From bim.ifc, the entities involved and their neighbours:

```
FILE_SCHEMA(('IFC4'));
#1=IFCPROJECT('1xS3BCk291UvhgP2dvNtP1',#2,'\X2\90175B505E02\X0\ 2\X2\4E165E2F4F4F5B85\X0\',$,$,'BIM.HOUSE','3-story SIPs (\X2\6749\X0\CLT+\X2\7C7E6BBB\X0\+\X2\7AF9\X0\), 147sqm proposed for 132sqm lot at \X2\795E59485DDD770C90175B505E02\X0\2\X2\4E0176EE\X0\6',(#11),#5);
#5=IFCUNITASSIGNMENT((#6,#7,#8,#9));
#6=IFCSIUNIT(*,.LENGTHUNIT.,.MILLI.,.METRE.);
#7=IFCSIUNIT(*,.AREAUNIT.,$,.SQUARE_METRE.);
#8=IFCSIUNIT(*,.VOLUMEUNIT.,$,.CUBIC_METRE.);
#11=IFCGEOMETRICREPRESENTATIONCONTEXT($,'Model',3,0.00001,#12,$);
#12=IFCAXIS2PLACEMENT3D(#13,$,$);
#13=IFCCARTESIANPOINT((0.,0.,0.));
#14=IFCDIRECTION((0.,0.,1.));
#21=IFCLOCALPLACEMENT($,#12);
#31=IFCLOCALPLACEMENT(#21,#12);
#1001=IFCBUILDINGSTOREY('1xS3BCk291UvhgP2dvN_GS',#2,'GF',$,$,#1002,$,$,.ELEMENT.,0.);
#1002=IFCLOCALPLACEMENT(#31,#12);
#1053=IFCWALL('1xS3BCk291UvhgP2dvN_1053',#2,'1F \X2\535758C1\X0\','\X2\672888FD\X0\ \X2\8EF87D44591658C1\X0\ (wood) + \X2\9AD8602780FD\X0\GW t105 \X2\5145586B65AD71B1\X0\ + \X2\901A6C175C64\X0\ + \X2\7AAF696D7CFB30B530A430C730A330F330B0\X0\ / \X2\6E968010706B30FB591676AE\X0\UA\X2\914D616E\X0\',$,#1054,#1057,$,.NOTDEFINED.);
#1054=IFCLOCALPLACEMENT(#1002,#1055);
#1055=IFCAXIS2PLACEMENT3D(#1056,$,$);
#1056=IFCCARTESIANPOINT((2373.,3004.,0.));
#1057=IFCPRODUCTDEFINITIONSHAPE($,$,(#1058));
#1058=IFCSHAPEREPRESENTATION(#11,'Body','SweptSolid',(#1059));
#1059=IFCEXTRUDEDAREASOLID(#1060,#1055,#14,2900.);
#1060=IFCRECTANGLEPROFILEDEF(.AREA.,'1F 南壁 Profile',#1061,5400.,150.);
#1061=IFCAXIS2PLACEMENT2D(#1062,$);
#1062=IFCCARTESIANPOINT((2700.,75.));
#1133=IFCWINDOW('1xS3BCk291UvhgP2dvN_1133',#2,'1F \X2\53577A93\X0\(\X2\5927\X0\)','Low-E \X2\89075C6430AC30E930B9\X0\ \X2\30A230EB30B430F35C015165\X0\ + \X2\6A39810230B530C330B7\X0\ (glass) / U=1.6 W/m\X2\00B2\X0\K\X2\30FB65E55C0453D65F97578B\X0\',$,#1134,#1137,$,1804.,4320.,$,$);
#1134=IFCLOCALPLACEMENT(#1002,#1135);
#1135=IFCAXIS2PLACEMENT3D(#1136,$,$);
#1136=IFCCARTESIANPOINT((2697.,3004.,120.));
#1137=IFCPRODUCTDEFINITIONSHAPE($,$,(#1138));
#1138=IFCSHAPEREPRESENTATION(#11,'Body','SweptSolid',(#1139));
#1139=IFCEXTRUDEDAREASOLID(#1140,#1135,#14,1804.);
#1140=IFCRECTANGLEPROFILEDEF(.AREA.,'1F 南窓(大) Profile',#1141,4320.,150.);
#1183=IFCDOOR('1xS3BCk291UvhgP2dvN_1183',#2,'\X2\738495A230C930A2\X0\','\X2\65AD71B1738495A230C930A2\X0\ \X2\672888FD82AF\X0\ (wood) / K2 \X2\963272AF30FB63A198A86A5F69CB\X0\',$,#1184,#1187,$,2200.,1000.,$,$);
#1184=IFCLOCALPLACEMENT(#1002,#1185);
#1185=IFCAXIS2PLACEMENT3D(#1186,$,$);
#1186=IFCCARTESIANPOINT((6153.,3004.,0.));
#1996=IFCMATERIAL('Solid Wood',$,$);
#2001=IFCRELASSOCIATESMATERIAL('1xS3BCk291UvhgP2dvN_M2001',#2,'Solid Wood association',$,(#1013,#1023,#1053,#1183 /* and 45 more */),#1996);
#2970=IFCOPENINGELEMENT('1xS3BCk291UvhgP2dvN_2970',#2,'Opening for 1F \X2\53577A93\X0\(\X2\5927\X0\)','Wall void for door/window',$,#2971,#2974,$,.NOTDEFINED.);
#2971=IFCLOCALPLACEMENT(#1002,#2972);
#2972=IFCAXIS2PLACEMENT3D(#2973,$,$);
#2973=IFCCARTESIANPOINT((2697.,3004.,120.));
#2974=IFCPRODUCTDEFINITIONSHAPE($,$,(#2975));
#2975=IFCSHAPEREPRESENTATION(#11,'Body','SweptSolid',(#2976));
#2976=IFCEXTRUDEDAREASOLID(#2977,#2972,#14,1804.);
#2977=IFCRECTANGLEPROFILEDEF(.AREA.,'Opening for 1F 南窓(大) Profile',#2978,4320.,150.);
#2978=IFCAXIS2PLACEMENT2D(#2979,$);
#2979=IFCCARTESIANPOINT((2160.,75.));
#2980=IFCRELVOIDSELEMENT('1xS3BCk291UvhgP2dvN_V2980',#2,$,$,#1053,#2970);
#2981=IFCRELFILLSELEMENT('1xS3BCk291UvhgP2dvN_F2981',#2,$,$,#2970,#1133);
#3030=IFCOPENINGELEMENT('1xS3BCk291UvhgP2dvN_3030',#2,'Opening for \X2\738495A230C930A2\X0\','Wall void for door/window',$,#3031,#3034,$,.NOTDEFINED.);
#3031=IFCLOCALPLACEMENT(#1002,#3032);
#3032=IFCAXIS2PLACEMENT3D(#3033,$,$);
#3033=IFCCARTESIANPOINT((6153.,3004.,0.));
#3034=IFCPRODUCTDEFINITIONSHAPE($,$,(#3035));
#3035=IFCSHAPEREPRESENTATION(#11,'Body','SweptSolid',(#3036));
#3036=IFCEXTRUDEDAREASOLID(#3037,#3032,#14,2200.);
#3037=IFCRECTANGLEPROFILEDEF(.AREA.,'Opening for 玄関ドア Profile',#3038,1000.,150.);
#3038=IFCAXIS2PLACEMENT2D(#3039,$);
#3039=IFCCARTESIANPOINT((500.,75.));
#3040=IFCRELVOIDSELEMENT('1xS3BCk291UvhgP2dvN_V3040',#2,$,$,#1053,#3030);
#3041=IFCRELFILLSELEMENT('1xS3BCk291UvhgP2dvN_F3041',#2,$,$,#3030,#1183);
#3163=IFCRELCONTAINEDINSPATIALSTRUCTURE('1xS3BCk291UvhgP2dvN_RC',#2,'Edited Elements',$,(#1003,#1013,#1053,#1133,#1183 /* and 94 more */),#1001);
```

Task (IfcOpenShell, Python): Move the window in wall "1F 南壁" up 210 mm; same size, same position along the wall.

```python
import numpy as np
import ifcopenshell
import ifcopenshell.api.geometry
import ifcopenshell.util.placement
import ifcopenshell.util.unit

model = ifcopenshell.open("bim.ifc")
unit_scale = ifcopenshell.util.unit.calculate_unit_scale(model)

window = model.by_id(1133)
opening = window.FillsVoids[0].RelatingOpeningElement
dz = 0.21 / unit_scale

shift = np.array([0.0, 0.0, dz])
# The window is not placed relative to its opening, so move both.
for product in (opening, window):
    matrix = ifcopenshell.util.placement.get_local_placement(product.ObjectPlacement)
    matrix[:3, 3] += shift
    ifcopenshell.api.geometry.edit_object_placement(model, product=product, matrix=matrix, is_si=False)

print(f"moved by {dz * unit_scale:+.3f} m")

model.write("bim-out.ifc")
```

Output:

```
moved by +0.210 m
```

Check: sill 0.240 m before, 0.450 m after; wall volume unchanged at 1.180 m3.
